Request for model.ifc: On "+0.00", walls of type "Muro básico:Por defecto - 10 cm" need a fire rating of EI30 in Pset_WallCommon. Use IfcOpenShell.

First a look at what the model holds.

```python
import ifcopenshell
import ifcopenshell.util.element

model = ifcopenshell.open("model.ifc")
print(model.schema)
storey = next(s for s in model.by_type("IfcBuildingStorey") if s.Name == "+0.00")
walls = [e for e in ifcopenshell.util.element.get_decomposition(storey) if e.is_a("IfcWall")]
seen = {}
for e in walls:
    element_type = ifcopenshell.util.element.get_type(e)
    key = (element_type.Name if element_type != e and element_type else None, ifcopenshell.util.element.get_pset(e, "Pset_WallCommon", "FireRating"))
    seen[key] = seen.get(key, 0) + 1
for (name, value), count in sorted(seen.items(), key=str):
    print(count, "x", name, "|", value)
```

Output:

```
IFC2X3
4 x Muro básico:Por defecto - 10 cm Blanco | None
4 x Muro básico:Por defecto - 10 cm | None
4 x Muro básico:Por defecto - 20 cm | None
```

```python
import ifcopenshell
import ifcopenshell.api.pset
import ifcopenshell.util.element

model = ifcopenshell.open("model.ifc")

storey = next(s for s in model.by_type("IfcBuildingStorey") if s.Name == "+0.00")
walls = [e for e in ifcopenshell.util.element.get_decomposition(storey) if e.is_a("IfcWall")]

count = 0
for e in walls:
    element_type = ifcopenshell.util.element.get_type(e)
    if element_type in (None, e) or element_type.Name != "Muro básico:Por defecto - 10 cm":
        continue
    # add_pset returns the element's existing set when there is one.
    pset = ifcopenshell.api.pset.add_pset(model, product=e, name="Pset_WallCommon")
    ifcopenshell.api.pset.edit_pset(model, pset=pset, properties={"FireRating": "EI30"})
    count += 1

print(count, "walls updated")

model.write("model_rev.ifc")
```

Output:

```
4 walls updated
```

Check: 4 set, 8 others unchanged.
